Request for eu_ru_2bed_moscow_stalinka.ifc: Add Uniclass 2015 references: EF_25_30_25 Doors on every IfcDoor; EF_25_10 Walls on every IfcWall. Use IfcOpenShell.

First a look at what the model holds.

```python
import ifcopenshell

model = ifcopenshell.open("eu_ru_2bed_moscow_stalinka.ifc")
print(model.schema)
print("classifications:", [c.Name for c in model.by_type("IfcClassification")])
for ifc_class in ("IfcDoor", "IfcRoof", "IfcStair", "IfcWall", "IfcWindow"):
    print(ifc_class, len(model.by_type(ifc_class)))
```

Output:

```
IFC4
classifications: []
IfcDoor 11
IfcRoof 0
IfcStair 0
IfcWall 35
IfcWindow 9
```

```python
import ifcopenshell
import ifcopenshell.api.classification

model = ifcopenshell.open("eu_ru_2bed_moscow_stalinka.ifc")

system = ifcopenshell.api.classification.add_classification(model, classification="Uniclass 2015")

codes = {
    "IfcDoor": ("EF_25_30_25", "Doors"),
    "IfcWall": ("EF_25_10", "Walls"),
}
for ifc_class, (code, name) in codes.items():
    products = model.by_type(ifc_class)
    ifcopenshell.api.classification.add_reference(
        model, products=products, classification=system, identification=code, name=name
    )
    print(code, len(products))

model.write("eu_ru_2bed_moscow_stalinka_edited.ifc")
```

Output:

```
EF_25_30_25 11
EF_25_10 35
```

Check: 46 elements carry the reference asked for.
